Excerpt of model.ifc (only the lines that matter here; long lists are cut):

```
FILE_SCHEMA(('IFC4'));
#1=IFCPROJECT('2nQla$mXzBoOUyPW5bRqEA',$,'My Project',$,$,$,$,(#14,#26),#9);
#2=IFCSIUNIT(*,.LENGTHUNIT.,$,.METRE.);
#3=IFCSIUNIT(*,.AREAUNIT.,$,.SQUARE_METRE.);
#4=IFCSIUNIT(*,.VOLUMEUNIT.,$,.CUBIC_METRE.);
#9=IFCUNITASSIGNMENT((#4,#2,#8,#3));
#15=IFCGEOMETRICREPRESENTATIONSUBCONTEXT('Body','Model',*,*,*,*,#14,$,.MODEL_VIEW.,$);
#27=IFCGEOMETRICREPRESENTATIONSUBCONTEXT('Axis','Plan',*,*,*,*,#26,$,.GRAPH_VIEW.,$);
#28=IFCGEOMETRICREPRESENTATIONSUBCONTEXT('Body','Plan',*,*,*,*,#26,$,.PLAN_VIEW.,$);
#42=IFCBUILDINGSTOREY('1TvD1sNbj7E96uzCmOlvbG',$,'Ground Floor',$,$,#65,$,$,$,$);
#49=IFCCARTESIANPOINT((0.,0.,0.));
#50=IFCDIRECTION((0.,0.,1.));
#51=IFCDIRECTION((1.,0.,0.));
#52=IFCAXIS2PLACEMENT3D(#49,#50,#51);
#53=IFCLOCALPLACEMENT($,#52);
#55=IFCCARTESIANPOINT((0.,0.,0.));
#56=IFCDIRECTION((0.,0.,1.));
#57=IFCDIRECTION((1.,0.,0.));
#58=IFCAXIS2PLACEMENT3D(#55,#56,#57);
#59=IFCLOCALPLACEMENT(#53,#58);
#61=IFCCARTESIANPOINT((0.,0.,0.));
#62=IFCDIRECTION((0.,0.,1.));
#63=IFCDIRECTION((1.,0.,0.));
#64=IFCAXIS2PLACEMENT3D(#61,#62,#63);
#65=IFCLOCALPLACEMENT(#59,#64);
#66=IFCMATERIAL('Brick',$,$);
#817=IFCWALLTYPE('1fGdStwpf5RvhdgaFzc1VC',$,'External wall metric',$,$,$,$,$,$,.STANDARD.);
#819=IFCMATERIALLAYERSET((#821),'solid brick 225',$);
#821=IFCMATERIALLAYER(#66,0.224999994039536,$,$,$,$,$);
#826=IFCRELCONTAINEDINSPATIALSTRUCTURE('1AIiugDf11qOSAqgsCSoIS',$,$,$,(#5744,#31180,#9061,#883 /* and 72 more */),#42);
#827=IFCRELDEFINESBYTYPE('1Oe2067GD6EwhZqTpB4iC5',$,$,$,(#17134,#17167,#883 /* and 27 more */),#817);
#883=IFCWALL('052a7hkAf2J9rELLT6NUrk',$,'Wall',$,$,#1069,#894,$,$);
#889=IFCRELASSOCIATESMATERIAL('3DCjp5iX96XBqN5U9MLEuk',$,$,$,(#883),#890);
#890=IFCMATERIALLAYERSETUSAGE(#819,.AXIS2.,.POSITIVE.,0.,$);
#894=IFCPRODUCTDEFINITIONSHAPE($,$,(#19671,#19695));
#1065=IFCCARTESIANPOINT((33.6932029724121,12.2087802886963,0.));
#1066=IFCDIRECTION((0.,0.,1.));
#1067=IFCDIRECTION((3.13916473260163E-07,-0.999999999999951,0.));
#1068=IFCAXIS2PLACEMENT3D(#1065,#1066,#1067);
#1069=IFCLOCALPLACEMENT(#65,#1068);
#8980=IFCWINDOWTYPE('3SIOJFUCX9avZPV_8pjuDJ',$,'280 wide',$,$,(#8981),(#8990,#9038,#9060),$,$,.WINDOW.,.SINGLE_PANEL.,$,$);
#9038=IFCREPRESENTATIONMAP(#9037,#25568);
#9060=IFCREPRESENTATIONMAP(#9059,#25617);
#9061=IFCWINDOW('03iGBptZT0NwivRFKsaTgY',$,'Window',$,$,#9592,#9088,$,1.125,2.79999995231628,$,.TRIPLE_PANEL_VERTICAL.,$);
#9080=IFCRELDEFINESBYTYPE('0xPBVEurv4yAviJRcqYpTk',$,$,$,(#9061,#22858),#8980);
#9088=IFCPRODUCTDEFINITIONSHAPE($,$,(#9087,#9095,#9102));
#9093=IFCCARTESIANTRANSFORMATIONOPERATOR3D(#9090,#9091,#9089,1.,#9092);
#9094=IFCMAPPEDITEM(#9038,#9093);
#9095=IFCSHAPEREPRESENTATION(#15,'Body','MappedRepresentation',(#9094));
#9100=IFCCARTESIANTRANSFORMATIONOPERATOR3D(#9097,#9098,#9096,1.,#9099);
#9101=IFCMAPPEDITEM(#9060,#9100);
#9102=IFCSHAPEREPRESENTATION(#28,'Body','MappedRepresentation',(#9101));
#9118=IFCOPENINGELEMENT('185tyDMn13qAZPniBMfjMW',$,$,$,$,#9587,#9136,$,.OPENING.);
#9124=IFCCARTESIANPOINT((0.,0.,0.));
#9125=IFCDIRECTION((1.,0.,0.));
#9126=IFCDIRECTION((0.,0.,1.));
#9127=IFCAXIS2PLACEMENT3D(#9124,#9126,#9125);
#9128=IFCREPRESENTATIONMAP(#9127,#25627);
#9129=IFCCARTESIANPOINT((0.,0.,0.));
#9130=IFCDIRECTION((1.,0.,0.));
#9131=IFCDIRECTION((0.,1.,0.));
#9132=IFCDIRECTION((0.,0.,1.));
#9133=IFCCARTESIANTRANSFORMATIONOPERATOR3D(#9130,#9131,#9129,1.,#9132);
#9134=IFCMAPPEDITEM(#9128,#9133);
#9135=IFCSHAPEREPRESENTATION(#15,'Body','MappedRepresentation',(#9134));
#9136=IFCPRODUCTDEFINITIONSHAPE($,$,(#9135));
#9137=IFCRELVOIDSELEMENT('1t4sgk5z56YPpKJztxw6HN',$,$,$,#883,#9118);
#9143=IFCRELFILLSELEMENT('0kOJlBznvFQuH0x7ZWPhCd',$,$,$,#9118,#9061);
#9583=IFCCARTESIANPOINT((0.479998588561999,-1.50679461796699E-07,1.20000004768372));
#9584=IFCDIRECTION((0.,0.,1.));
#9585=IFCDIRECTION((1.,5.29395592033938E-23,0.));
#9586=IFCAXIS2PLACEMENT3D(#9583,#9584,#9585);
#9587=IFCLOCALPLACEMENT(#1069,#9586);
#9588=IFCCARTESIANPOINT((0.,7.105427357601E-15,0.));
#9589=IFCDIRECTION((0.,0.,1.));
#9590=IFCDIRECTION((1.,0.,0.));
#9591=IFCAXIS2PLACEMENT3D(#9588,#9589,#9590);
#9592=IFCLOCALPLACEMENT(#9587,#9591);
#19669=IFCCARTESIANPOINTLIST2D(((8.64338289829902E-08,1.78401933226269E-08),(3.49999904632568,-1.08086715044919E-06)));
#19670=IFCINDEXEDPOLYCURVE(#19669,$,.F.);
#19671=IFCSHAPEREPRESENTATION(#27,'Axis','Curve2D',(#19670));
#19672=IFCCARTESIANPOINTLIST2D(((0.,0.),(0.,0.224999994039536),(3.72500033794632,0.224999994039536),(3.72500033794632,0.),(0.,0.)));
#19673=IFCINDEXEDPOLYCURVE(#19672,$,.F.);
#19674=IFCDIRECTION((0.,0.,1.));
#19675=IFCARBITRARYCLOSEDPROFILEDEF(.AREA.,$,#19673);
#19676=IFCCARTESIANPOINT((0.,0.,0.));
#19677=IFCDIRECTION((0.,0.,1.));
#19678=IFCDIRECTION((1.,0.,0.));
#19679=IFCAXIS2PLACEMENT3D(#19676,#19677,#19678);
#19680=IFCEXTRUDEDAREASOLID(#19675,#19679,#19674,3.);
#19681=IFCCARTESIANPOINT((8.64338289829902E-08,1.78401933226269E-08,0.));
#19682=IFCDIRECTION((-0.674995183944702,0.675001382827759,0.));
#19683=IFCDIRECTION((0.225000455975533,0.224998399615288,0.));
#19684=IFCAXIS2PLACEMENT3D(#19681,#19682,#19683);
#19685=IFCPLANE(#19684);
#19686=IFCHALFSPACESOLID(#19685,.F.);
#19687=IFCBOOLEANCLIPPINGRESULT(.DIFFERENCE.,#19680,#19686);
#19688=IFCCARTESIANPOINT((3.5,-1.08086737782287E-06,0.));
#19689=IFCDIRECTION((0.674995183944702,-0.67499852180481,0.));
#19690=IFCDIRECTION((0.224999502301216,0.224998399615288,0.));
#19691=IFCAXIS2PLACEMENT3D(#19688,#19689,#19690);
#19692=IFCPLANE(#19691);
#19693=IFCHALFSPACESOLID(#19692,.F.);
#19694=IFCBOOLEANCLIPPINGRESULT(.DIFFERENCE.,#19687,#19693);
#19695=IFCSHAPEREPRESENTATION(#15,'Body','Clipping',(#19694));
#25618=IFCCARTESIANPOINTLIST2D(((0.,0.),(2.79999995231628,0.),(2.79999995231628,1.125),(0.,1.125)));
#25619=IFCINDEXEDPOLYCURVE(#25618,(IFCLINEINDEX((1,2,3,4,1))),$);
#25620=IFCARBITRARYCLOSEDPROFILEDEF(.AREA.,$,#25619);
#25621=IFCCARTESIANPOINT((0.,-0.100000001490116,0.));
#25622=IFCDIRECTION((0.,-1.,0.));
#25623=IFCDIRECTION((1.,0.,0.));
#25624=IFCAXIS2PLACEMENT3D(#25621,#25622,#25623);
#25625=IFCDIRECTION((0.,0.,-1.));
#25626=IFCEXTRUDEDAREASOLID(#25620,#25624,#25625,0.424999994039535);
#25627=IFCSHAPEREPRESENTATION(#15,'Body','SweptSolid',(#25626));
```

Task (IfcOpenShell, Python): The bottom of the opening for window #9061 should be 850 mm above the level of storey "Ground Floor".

```python
import numpy as np
import ifcopenshell
import ifcopenshell.api.geometry
import ifcopenshell.geom
import ifcopenshell.util.element
import ifcopenshell.util.placement
import ifcopenshell.util.shape
import ifcopenshell.util.unit

model = ifcopenshell.open("model.ifc")
unit_scale = ifcopenshell.util.unit.calculate_unit_scale(model)

window = model.by_id(9061)
opening = window.FillsVoids[0].RelatingOpeningElement
storey = ifcopenshell.util.element.get_container(window, ifc_class="IfcBuildingStorey")
level = ifcopenshell.util.placement.get_local_placement(storey.ObjectPlacement)[2, 3]

# The opening's origin need not be at the sill, so measure its lowest point.
shape = ifcopenshell.geom.create_shape(ifcopenshell.geom.settings(), opening)
bottom = ifcopenshell.util.shape.get_shape_bottom_elevation(shape, shape.geometry) / unit_scale
dz = level + 0.85 - bottom

shift = np.array([0.0, 0.0, dz])
# The window is placed relative to its opening, so it follows when the opening moves.
matrix = ifcopenshell.util.placement.get_local_placement(opening.ObjectPlacement)
matrix[:3, 3] += shift
ifcopenshell.api.geometry.edit_object_placement(
    model, product=opening, matrix=matrix, is_si=False, should_transform_children=True
)

print(f"moved by {dz * unit_scale:+.3f} m")

model.write("model_edited.ifc")
```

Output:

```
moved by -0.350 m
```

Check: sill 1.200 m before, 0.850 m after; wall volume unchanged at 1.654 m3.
